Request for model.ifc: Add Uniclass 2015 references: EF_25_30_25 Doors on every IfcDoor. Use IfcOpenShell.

First a look at what the model holds.

```python
import ifcopenshell

model = ifcopenshell.open("model.ifc")
print(model.schema)
print("classifications:", [c.Name for c in model.by_type("IfcClassification")])
for ifc_class in ("IfcDoor", "IfcRoof", "IfcStair", "IfcWall", "IfcWindow"):
    print(ifc_class, len(model.by_type(ifc_class)))
```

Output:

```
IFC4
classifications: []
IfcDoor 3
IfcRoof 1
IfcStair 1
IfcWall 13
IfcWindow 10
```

```python
import ifcopenshell
import ifcopenshell.api.classification

model = ifcopenshell.open("model.ifc")

system = ifcopenshell.api.classification.add_classification(model, classification="Uniclass 2015")

codes = {
    "IfcDoor": ("EF_25_30_25", "Doors"),
}
for ifc_class, (code, name) in codes.items():
    products = model.by_type(ifc_class)
    ifcopenshell.api.classification.add_reference(
        model, products=products, classification=system, identification=code, name=name
    )
    print(code, len(products))

model.write("model_v2.ifc")
```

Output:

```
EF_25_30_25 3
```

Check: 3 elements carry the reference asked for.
